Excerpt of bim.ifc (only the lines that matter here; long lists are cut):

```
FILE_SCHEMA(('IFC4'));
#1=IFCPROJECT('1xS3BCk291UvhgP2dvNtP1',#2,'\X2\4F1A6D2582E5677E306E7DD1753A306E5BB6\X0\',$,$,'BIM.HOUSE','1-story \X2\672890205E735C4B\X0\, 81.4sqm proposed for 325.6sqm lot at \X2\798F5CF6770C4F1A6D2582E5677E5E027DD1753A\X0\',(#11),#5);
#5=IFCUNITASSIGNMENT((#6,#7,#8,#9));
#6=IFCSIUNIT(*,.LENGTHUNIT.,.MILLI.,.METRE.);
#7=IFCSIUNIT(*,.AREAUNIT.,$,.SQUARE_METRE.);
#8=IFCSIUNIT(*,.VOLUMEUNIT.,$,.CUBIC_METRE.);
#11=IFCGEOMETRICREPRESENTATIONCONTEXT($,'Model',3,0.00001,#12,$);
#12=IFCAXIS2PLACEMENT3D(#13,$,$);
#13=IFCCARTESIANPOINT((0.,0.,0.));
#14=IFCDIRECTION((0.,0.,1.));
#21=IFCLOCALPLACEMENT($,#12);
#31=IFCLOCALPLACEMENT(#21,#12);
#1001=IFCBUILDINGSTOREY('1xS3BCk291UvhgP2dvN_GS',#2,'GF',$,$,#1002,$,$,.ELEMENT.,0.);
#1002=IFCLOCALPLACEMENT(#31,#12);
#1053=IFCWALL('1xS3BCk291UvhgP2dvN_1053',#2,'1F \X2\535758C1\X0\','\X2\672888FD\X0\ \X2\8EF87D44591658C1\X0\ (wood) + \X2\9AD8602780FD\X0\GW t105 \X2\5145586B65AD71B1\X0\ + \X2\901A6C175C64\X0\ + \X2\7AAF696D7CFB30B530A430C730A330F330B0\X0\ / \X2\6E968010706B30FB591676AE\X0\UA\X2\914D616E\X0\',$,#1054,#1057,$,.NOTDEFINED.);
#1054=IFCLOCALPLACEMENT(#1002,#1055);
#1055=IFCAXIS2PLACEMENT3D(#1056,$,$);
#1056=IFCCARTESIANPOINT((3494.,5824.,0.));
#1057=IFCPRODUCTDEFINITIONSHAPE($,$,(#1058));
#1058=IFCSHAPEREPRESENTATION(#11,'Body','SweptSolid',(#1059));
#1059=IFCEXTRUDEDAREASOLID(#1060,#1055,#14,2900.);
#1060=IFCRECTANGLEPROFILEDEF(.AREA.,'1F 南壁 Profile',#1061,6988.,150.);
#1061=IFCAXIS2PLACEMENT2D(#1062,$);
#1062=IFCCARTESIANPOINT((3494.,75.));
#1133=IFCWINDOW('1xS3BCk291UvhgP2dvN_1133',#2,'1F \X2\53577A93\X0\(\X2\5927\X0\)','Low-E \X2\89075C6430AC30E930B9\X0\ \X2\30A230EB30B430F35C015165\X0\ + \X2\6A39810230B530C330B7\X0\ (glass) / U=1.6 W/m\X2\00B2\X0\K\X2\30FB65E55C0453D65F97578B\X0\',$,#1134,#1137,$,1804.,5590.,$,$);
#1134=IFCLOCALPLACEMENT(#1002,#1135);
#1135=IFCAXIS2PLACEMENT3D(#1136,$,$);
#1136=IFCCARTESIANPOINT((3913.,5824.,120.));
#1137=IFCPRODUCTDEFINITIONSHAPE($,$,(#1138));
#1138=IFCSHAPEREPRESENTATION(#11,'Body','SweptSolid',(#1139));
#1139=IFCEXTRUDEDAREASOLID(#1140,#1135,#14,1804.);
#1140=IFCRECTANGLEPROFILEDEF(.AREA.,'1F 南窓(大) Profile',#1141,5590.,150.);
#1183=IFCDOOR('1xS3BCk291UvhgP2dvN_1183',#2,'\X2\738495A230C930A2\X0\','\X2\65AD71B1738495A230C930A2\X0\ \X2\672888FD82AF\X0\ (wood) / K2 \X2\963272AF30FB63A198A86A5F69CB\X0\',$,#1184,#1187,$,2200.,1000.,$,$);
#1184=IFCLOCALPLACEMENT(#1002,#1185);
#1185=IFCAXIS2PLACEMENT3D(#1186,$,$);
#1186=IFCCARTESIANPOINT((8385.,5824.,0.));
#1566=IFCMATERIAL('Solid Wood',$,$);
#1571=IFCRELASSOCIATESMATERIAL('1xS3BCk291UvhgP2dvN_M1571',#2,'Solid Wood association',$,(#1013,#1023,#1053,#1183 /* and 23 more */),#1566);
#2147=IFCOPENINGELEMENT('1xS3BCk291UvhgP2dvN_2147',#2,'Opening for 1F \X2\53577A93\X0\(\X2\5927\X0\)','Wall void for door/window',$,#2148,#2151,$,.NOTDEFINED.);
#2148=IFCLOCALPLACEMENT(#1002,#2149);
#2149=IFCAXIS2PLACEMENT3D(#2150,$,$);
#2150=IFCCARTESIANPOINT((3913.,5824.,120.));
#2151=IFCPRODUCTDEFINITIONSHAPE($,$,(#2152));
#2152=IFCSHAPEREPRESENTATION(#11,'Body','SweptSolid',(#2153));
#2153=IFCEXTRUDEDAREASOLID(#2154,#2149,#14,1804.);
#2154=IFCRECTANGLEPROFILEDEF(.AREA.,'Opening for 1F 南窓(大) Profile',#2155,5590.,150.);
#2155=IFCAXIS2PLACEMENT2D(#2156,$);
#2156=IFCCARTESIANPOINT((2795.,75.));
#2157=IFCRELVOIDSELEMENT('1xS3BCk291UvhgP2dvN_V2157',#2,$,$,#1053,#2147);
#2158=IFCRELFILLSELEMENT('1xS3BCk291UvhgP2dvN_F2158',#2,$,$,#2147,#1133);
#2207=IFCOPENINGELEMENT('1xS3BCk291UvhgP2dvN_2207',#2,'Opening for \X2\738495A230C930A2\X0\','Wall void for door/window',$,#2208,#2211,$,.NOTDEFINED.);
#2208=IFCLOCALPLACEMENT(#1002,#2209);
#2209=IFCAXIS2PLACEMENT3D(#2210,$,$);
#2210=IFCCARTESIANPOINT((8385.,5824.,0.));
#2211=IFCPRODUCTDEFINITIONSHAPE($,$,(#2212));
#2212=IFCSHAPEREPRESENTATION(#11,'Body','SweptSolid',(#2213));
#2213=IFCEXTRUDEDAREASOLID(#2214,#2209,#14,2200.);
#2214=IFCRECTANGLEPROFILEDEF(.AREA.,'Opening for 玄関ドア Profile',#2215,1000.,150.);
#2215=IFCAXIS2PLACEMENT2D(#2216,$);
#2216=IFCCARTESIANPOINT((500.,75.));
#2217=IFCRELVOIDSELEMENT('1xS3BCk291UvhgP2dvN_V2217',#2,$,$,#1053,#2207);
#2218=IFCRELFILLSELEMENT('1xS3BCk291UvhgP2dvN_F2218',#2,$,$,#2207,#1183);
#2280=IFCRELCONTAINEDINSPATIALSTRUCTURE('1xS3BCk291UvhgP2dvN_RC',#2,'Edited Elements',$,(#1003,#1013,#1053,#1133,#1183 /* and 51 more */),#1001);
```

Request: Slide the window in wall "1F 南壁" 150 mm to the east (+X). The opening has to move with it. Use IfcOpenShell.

```python
import ifcopenshell
import ifcopenshell.api.geometry
import ifcopenshell.util.placement
import ifcopenshell.util.unit

model = ifcopenshell.open("bim.ifc")
unit_scale = ifcopenshell.util.unit.calculate_unit_scale(model)

window = model.by_guid("1xS3BCk291UvhgP2dvN_1133")
opening = window.FillsVoids[0].RelatingOpeningElement
wall = opening.VoidsElements[0].RelatingBuildingElement

wall_matrix = ifcopenshell.util.placement.get_local_placement(wall.ObjectPlacement)
shift = wall_matrix[:3, 0] * 0.15 / unit_scale
before = ifcopenshell.util.placement.get_local_placement(window.ObjectPlacement)[:3, 3].copy()

# The window is not placed relative to its opening, so move both.
for product in (opening, window):
    matrix = ifcopenshell.util.placement.get_local_placement(product.ObjectPlacement)
    matrix[:3, 3] += shift
    ifcopenshell.api.geometry.edit_object_placement(model, product=product, matrix=matrix, is_si=False)

after = ifcopenshell.util.placement.get_local_placement(window.ObjectPlacement)[:3, 3]
print("window moved by", (after - before).round(3) + 0.0)

model.write("bim_rev.ifc")
```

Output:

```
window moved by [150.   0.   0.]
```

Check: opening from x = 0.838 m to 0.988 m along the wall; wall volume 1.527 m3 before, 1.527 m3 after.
